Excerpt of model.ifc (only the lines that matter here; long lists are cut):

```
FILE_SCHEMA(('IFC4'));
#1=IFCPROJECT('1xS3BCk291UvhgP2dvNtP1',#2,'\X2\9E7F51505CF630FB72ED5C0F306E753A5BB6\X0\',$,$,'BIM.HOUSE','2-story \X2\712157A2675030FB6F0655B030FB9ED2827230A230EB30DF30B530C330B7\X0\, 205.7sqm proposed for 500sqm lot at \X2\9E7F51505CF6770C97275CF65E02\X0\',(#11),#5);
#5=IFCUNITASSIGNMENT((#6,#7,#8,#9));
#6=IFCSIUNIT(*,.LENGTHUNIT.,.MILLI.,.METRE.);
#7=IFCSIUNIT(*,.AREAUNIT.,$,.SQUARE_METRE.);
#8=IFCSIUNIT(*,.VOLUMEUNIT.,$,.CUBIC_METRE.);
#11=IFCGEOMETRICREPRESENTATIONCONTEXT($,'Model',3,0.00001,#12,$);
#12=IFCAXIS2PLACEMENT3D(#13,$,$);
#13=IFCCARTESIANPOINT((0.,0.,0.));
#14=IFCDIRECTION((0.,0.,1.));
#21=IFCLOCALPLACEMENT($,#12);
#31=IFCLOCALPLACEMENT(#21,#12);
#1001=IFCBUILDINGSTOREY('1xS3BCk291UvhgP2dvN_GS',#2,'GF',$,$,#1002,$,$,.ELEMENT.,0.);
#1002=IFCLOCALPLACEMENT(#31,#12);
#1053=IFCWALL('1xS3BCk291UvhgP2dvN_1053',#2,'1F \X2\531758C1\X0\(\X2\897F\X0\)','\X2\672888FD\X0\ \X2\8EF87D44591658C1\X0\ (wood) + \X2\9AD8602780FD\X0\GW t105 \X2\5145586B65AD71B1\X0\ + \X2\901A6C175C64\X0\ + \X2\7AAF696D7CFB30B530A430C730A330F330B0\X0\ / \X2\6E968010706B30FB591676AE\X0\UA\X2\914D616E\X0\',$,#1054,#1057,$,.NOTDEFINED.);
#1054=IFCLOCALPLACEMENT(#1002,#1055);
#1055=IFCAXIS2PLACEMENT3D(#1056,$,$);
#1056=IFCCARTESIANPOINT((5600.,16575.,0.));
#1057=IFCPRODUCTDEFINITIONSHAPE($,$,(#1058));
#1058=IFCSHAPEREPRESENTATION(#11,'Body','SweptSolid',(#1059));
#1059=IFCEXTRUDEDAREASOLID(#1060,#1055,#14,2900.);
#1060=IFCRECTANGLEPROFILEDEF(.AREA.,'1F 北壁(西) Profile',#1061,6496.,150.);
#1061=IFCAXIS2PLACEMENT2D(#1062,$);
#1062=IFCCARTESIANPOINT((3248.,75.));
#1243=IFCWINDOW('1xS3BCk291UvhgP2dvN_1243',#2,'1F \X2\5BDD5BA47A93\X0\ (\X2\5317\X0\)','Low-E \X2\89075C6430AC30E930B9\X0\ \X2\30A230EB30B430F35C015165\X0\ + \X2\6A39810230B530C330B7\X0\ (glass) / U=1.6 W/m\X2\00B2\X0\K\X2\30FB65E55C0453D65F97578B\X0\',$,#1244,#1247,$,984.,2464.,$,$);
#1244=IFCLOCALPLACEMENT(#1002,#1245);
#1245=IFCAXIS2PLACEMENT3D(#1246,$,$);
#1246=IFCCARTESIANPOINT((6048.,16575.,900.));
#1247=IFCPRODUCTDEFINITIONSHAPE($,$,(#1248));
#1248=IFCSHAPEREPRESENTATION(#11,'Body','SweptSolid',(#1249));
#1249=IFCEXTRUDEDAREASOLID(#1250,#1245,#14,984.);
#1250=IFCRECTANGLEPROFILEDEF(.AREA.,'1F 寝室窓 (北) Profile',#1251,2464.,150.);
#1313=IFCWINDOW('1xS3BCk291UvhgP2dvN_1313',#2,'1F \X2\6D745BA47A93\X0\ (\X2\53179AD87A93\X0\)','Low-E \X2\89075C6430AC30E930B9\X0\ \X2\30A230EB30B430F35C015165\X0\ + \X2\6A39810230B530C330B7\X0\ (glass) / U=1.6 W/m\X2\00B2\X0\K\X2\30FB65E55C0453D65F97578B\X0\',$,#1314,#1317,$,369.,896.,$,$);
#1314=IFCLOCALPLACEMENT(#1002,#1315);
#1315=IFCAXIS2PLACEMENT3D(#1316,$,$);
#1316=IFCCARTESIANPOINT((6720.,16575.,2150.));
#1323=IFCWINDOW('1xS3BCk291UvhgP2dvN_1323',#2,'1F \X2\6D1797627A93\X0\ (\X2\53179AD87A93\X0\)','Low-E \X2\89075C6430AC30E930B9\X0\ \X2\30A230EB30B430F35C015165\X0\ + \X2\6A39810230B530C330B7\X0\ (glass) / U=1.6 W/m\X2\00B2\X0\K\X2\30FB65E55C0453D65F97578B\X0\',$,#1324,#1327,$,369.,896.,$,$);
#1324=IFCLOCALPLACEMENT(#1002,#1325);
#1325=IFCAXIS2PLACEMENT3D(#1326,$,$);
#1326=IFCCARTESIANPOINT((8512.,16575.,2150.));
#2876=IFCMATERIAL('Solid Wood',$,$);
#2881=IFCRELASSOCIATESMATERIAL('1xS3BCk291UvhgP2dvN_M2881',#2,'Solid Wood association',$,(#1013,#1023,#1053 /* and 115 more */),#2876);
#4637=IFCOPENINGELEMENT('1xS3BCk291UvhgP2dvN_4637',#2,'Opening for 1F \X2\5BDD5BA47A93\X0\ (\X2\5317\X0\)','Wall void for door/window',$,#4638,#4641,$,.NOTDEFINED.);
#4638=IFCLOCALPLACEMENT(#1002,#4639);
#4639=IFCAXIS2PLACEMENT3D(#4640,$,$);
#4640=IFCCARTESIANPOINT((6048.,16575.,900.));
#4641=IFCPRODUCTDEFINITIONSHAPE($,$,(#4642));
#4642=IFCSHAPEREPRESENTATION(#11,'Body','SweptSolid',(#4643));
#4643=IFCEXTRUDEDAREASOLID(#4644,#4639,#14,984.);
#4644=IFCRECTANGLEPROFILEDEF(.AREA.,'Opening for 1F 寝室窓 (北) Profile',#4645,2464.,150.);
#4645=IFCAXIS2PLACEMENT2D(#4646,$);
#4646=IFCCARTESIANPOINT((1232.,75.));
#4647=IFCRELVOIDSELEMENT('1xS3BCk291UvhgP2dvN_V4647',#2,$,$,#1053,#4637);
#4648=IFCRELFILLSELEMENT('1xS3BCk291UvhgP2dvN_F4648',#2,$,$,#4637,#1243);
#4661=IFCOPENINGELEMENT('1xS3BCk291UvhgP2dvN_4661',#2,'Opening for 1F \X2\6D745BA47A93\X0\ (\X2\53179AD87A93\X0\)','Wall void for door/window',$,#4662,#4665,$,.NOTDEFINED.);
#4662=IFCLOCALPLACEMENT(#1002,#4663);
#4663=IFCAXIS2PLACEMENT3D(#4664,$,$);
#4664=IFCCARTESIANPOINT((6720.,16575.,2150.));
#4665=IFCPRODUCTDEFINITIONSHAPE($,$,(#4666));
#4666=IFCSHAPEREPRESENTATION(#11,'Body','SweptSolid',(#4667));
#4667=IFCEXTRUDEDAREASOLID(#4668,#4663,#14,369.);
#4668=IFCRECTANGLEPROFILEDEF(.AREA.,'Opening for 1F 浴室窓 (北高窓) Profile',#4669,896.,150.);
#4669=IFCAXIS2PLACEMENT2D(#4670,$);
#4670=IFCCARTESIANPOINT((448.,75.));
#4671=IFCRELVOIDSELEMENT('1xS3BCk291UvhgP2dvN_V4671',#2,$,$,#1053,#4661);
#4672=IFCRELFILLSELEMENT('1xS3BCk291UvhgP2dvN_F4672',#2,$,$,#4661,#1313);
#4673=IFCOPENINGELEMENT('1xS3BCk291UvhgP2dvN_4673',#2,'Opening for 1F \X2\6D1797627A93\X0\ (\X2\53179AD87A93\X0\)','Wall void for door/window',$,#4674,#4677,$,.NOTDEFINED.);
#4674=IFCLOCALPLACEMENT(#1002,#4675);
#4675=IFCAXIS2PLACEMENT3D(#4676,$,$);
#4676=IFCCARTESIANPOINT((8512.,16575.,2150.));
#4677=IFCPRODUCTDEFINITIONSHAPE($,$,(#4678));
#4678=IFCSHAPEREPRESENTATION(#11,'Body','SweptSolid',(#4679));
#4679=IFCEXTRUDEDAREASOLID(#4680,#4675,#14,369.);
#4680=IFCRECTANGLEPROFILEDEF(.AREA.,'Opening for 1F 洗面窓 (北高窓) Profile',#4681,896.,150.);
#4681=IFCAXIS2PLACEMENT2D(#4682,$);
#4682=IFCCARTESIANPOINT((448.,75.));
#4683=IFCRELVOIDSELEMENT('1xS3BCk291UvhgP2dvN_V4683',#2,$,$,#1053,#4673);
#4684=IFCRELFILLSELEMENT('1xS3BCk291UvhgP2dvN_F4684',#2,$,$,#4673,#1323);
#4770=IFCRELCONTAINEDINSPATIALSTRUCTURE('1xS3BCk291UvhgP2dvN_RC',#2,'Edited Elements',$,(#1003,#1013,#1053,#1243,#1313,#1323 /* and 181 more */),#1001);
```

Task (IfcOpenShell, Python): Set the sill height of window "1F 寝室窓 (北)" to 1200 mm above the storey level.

```python
import numpy as np
import ifcopenshell
import ifcopenshell.api.geometry
import ifcopenshell.geom
import ifcopenshell.util.element
import ifcopenshell.util.placement
import ifcopenshell.util.shape
import ifcopenshell.util.unit

model = ifcopenshell.open("model.ifc")
unit_scale = ifcopenshell.util.unit.calculate_unit_scale(model)

window = model.by_guid("1xS3BCk291UvhgP2dvN_1243")
opening = window.FillsVoids[0].RelatingOpeningElement
storey = ifcopenshell.util.element.get_container(window, ifc_class="IfcBuildingStorey")
level = ifcopenshell.util.placement.get_local_placement(storey.ObjectPlacement)[2, 3]

# The opening's origin need not be at the sill, so measure its lowest point.
shape = ifcopenshell.geom.create_shape(ifcopenshell.geom.settings(), opening)
bottom = ifcopenshell.util.shape.get_shape_bottom_elevation(shape, shape.geometry) / unit_scale
dz = level + 1.2 / unit_scale - bottom

shift = np.array([0.0, 0.0, dz])
# The window is not placed relative to its opening, so move both.
for product in (opening, window):
    matrix = ifcopenshell.util.placement.get_local_placement(product.ObjectPlacement)
    matrix[:3, 3] += shift
    ifcopenshell.api.geometry.edit_object_placement(model, product=product, matrix=matrix, is_si=False)

print(f"moved by {dz * unit_scale:+.3f} m")

model.write("model_edited.ifc")
```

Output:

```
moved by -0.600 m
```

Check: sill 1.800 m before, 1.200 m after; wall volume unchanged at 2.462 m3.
